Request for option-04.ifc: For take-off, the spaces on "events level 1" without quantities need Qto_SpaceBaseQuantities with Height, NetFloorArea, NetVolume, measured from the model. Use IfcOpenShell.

First a look at what the model holds.

```python
import ifcopenshell
import ifcopenshell.util.element
import ifcopenshell.util.unit

model = ifcopenshell.open("option-04.ifc")
print(model.schema)
for unit_type in ("LENGTHUNIT", "AREAUNIT", "VOLUMEUNIT"):
    print(unit_type, ifcopenshell.util.unit.calculate_unit_scale(model, unit_type))
storey = next(s for s in model.by_type("IfcBuildingStorey") if s.Name == "events level 1")
spaces = [e for e in ifcopenshell.util.element.get_decomposition(storey) if e.is_a("IfcSpace")]
for e in sorted(spaces, key=lambda e: e.id()):
    print(e.id(), e.is_a(), e.Name, list(ifcopenshell.util.element.get_psets(e, qtos_only=True)), sep=" | ")
```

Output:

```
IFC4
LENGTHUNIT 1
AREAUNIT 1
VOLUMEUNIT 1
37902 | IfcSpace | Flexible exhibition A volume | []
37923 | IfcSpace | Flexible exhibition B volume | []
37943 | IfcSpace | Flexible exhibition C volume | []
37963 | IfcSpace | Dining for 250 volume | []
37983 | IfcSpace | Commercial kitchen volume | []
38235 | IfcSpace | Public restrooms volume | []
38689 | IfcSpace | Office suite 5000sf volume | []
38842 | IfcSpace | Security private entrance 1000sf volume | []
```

```python
import ifcopenshell
import ifcopenshell.api.pset
import ifcopenshell.geom
import ifcopenshell.util.element
import ifcopenshell.util.shape
import ifcopenshell.util.unit

model = ifcopenshell.open("option-04.ifc")
unit_scale = ifcopenshell.util.unit.calculate_unit_scale(model)
area_scale = ifcopenshell.util.unit.calculate_unit_scale(model, "AREAUNIT")
volume_scale = ifcopenshell.util.unit.calculate_unit_scale(model, "VOLUMEUNIT")
settings = ifcopenshell.geom.settings()

storey = next(s for s in model.by_type("IfcBuildingStorey") if s.Name == "events level 1")
spaces = [e for e in ifcopenshell.util.element.get_decomposition(storey) if e.is_a("IfcSpace")]

for e in sorted(spaces, key=lambda e: e.id()):
    if ifcopenshell.util.element.get_psets(e, qtos_only=True, should_inherit=False):
        continue
    # Geometry comes back in metres, in the element's own axes.
    shape = ifcopenshell.geom.create_shape(settings, e)
    values = {
        "Height": ifcopenshell.util.shape.get_z(shape.geometry) / unit_scale,
        "NetFloorArea": ifcopenshell.util.shape.get_footprint_area(shape.geometry) / area_scale,
        "NetVolume": ifcopenshell.util.shape.get_volume(shape.geometry) / volume_scale,
    }
    qto = ifcopenshell.api.pset.add_qto(model, product=e, name="Qto_SpaceBaseQuantities")
    ifcopenshell.api.pset.edit_qto(model, qto=qto, properties=values)
    print(e.id(), {k: round(v, 3) for k, v in values.items()})

model.write("option-04_edited.ifc")
```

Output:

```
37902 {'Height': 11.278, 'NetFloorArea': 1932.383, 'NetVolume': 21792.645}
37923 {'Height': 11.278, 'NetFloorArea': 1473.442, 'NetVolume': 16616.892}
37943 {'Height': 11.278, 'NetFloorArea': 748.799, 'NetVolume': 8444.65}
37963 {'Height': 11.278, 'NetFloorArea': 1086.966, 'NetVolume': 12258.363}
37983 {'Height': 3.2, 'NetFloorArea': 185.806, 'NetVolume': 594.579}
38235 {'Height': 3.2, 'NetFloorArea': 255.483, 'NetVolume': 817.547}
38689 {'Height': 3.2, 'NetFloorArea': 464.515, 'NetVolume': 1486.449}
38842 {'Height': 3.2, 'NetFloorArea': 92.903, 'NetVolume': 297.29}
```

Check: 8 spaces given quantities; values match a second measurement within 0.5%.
